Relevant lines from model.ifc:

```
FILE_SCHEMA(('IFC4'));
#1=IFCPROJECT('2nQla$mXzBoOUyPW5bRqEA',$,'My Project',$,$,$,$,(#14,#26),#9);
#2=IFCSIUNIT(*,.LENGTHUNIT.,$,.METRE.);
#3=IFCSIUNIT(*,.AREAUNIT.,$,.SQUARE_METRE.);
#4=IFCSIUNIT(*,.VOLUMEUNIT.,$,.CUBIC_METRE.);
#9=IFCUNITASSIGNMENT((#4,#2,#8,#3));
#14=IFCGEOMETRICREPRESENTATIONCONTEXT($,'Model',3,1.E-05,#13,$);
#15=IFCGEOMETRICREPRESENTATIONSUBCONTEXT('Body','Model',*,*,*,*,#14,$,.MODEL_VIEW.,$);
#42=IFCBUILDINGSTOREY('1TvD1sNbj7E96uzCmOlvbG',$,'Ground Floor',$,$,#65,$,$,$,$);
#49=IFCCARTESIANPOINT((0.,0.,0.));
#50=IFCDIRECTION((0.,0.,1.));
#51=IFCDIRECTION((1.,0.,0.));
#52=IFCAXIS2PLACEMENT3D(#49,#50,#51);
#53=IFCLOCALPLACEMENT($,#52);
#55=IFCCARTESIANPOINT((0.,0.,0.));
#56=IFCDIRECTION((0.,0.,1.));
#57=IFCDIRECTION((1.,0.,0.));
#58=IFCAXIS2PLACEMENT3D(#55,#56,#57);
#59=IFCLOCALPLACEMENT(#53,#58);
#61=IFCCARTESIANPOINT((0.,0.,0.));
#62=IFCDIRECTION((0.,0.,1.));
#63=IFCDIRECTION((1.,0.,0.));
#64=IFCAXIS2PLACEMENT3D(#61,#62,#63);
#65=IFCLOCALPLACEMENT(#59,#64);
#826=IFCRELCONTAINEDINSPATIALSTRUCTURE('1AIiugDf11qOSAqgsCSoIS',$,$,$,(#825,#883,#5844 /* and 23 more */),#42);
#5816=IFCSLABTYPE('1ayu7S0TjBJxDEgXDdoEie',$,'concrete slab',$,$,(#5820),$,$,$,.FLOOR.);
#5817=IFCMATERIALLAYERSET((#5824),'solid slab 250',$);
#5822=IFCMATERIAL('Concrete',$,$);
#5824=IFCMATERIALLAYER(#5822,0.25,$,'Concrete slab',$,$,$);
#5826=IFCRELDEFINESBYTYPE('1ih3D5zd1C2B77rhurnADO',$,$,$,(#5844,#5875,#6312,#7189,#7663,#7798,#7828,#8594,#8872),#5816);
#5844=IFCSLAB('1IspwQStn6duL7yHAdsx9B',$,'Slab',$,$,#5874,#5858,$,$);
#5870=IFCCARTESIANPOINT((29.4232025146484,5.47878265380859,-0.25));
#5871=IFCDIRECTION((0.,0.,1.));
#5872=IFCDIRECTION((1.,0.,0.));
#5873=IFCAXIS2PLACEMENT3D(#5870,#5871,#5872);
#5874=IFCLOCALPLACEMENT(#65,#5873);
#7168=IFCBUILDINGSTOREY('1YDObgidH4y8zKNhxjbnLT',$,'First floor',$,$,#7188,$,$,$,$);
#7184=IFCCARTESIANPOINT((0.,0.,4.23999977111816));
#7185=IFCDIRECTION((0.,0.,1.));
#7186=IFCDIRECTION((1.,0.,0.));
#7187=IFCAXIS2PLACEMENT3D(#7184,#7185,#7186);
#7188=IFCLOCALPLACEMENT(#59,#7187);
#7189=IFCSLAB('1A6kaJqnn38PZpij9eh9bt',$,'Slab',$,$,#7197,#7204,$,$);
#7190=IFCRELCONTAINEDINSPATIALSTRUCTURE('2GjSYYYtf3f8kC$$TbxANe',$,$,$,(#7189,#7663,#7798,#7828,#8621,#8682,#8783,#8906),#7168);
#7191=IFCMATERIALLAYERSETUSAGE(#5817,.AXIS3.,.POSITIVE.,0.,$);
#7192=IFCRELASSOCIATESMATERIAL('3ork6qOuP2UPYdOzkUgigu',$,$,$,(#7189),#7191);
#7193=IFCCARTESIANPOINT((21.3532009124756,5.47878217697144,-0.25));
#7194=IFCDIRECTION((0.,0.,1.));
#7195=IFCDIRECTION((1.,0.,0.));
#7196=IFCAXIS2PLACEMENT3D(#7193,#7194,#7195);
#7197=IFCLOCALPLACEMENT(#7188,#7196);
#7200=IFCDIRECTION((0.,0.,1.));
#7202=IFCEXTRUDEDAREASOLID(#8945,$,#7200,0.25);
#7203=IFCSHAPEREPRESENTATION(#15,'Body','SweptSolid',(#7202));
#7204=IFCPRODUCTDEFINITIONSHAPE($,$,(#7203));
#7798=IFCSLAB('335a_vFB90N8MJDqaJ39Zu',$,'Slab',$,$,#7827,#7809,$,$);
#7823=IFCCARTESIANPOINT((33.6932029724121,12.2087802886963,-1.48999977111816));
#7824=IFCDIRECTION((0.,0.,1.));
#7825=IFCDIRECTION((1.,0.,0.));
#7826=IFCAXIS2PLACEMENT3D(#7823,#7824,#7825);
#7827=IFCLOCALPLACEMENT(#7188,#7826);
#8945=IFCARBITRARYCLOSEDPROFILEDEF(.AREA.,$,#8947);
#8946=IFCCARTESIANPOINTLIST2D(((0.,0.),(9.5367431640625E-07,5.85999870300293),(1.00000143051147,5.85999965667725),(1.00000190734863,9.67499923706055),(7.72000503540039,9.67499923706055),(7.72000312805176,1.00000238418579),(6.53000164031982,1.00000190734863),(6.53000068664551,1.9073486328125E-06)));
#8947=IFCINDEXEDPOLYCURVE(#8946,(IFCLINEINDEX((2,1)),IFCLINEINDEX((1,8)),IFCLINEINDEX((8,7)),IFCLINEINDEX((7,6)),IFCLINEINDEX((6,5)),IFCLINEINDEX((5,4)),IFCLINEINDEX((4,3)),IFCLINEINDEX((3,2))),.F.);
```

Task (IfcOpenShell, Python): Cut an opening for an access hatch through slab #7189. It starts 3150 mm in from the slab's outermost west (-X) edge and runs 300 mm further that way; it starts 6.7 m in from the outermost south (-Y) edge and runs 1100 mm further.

```python
import numpy as np
import ifcopenshell
import ifcopenshell.api.feature
import ifcopenshell.api.geometry
import ifcopenshell.api.root
import ifcopenshell.geom
import ifcopenshell.util.placement
import ifcopenshell.util.representation
import ifcopenshell.util.shape
import ifcopenshell.util.unit

model = ifcopenshell.open("model.ifc")
unit_scale = ifcopenshell.util.unit.calculate_unit_scale(model)
settings = ifcopenshell.geom.settings()


def volume(element):
    """Net volume in cubic metres, openings subtracted."""
    shape = ifcopenshell.geom.create_shape(settings, element)
    return ifcopenshell.util.shape.get_volume(shape.geometry)


slab = model.by_guid("1A6kaJqnn38PZpij9eh9bt")
before = volume(slab)

# Extent in the slab's own axes, in metres. The edges named are its -X and -Y sides.
slab_shape = ifcopenshell.geom.create_shape(settings, slab)
vertices = ifcopenshell.util.shape.get_vertices(slab_shape.geometry)
x_min, y_min, bottom = vertices.min(axis=0)
top = vertices[:, 2].max()

opening = ifcopenshell.api.root.create_entity(model, ifc_class="IfcOpeningElement", name="Access hatch opening", predefined_type="OPENING")
context = ifcopenshell.util.representation.get_context(model, "Model", "Body", "MODEL_VIEW")
width, depth = 0.3, 1.1
outline = [(0.0, 0.0), (width, 0.0), (width, depth), (0.0, depth), (0.0, 0.0)]
# Overshoot both faces by 50 mm so the cut is clean.
shape = ifcopenshell.api.geometry.add_slab_representation(
    model, context=context, depth=top - bottom + 0.1, polyline=outline
)
ifcopenshell.api.geometry.assign_representation(model, product=opening, representation=shape)

matrix = ifcopenshell.util.placement.get_local_placement(slab.ObjectPlacement)
matrix[:, 3] = matrix @ np.append(np.array([x_min + 3.15, y_min + 6.7, bottom - 0.05]) / unit_scale, 1.0)
ifcopenshell.api.geometry.edit_object_placement(model, product=opening, matrix=matrix, is_si=False)
ifcopenshell.api.feature.add_feature(model, feature=opening, element=slab)

after = volume(slab)

print(f"slab volume {before:.3f} -> {after:.3f} m3")

model.write("model_updated.ifc")
```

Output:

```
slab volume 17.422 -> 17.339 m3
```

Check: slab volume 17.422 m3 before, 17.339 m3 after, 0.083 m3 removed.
